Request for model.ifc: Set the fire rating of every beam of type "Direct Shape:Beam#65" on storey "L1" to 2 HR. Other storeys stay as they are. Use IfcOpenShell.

First a look at what the model holds.

```python
import ifcopenshell
import ifcopenshell.util.element

model = ifcopenshell.open("model.ifc")
print(model.schema)
storey = next(s for s in model.by_type("IfcBuildingStorey") if s.Name == "L1")
beams = [e for e in ifcopenshell.util.element.get_decomposition(storey) if e.is_a("IfcBeam")]
seen = {}
for e in beams:
    element_type = ifcopenshell.util.element.get_type(e)
    key = (element_type.Name if element_type != e and element_type else None, ifcopenshell.util.element.get_pset(e, "Pset_BeamCommon", "FireRating"))
    seen[key] = seen.get(key, 0) + 1
for (name, value), count in sorted(seen.items(), key=str):
    print(count, "x", name, "|", value)
```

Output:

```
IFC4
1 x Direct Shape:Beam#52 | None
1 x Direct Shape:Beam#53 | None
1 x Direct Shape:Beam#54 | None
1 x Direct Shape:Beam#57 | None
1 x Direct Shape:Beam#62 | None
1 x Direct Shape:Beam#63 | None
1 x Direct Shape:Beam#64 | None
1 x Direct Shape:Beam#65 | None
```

```python
import ifcopenshell
import ifcopenshell.api.pset
import ifcopenshell.util.element

model = ifcopenshell.open("model.ifc")

storey = next(s for s in model.by_type("IfcBuildingStorey") if s.Name == "L1")
beams = [e for e in ifcopenshell.util.element.get_decomposition(storey) if e.is_a("IfcBeam")]

count = 0
for e in beams:
    element_type = ifcopenshell.util.element.get_type(e)
    if element_type in (None, e) or element_type.Name != "Direct Shape:Beam#65":
        continue
    # add_pset returns the element's existing set when there is one.
    pset = ifcopenshell.api.pset.add_pset(model, product=e, name="Pset_BeamCommon")
    ifcopenshell.api.pset.edit_pset(model, pset=pset, properties={"FireRating": "2 HR"})
    count += 1

print(count, "beams updated")

model.write("model_edited.ifc")
```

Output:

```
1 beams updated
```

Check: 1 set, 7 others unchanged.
